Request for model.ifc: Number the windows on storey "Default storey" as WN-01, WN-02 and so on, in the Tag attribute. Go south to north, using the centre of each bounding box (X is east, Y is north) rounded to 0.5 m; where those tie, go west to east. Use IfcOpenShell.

First a look at what the model holds.

```python
import ifcopenshell
import ifcopenshell.util.element
import ifcopenshell.util.placement

model = ifcopenshell.open("model.ifc")
print(model.schema)
storey = next(s for s in model.by_type("IfcBuildingStorey") if s.Name == "Default storey")
windows = [e for e in ifcopenshell.util.element.get_decomposition(storey) if e.is_a("IfcWindow")]
for e in sorted(windows, key=lambda e: e.id()):
    origin = ifcopenshell.util.placement.get_local_placement(e.ObjectPlacement)[:3, 3]
    print(e.id(), e.Tag, e.Name, origin.round(2) + 0.0, sep=" | ")
```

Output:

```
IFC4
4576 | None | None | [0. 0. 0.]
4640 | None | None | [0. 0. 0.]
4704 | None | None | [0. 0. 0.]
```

```python
import ifcopenshell
import ifcopenshell.geom
import ifcopenshell.util.element
import ifcopenshell.util.shape

model = ifcopenshell.open("model.ifc")
settings = ifcopenshell.geom.settings()
settings.set("use-world-coords", True)


def centre(element):
    shape = ifcopenshell.geom.create_shape(settings, element)
    return ifcopenshell.util.shape.get_bbox_centroid(shape.geometry)


storey = next(s for s in model.by_type("IfcBuildingStorey") if s.Name == "Default storey")
windows = [e for e in ifcopenshell.util.element.get_decomposition(storey) if e.is_a("IfcWindow")]

# Insertion points can sit at a corner or the storey origin, so sort by the geometry (in metres).
centres = {e: centre(e) for e in windows}
windows.sort(key=lambda e: (round(centres[e][1] / 0.5), centres[e][0]))

for i, e in enumerate(windows, start=1):
    number = f"WN-{i:02d}"
    e.Tag = number
    print(e.id(), number)

model.write("model_edited.ifc")
```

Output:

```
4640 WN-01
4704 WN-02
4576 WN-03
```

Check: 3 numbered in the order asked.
